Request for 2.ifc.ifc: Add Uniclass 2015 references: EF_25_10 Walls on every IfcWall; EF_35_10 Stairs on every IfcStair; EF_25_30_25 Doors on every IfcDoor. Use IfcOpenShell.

First a look at what the model holds.

```python
import ifcopenshell

model = ifcopenshell.open("2.ifc.ifc")
print(model.schema)
print("classifications:", [c.Name for c in model.by_type("IfcClassification")])
for ifc_class in ("IfcDoor", "IfcRoof", "IfcStair", "IfcWall", "IfcWindow"):
    print(ifc_class, len(model.by_type(ifc_class)))
```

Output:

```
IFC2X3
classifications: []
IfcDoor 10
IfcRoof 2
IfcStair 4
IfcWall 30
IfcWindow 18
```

```python
import ifcopenshell
import ifcopenshell.api.classification

model = ifcopenshell.open("2.ifc.ifc")

# IFC2X3 requires Source and Edition and has no link from the project to the system.
system = model.create_entity("IfcClassification", Source="NBS", Edition="2015", Name="Uniclass 2015")

codes = {
    "IfcWall": ("EF_25_10", "Walls"),
    "IfcStair": ("EF_35_10", "Stairs"),
    "IfcDoor": ("EF_25_30_25", "Doors"),
}
for ifc_class, (code, name) in codes.items():
    products = model.by_type(ifc_class)
    ifcopenshell.api.classification.add_reference(
        model, products=products, classification=system, identification=code, name=name
    )
    print(code, len(products))

model.write("2.ifc-out.ifc")
```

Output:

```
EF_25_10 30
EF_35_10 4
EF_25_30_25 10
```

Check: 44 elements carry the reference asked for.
